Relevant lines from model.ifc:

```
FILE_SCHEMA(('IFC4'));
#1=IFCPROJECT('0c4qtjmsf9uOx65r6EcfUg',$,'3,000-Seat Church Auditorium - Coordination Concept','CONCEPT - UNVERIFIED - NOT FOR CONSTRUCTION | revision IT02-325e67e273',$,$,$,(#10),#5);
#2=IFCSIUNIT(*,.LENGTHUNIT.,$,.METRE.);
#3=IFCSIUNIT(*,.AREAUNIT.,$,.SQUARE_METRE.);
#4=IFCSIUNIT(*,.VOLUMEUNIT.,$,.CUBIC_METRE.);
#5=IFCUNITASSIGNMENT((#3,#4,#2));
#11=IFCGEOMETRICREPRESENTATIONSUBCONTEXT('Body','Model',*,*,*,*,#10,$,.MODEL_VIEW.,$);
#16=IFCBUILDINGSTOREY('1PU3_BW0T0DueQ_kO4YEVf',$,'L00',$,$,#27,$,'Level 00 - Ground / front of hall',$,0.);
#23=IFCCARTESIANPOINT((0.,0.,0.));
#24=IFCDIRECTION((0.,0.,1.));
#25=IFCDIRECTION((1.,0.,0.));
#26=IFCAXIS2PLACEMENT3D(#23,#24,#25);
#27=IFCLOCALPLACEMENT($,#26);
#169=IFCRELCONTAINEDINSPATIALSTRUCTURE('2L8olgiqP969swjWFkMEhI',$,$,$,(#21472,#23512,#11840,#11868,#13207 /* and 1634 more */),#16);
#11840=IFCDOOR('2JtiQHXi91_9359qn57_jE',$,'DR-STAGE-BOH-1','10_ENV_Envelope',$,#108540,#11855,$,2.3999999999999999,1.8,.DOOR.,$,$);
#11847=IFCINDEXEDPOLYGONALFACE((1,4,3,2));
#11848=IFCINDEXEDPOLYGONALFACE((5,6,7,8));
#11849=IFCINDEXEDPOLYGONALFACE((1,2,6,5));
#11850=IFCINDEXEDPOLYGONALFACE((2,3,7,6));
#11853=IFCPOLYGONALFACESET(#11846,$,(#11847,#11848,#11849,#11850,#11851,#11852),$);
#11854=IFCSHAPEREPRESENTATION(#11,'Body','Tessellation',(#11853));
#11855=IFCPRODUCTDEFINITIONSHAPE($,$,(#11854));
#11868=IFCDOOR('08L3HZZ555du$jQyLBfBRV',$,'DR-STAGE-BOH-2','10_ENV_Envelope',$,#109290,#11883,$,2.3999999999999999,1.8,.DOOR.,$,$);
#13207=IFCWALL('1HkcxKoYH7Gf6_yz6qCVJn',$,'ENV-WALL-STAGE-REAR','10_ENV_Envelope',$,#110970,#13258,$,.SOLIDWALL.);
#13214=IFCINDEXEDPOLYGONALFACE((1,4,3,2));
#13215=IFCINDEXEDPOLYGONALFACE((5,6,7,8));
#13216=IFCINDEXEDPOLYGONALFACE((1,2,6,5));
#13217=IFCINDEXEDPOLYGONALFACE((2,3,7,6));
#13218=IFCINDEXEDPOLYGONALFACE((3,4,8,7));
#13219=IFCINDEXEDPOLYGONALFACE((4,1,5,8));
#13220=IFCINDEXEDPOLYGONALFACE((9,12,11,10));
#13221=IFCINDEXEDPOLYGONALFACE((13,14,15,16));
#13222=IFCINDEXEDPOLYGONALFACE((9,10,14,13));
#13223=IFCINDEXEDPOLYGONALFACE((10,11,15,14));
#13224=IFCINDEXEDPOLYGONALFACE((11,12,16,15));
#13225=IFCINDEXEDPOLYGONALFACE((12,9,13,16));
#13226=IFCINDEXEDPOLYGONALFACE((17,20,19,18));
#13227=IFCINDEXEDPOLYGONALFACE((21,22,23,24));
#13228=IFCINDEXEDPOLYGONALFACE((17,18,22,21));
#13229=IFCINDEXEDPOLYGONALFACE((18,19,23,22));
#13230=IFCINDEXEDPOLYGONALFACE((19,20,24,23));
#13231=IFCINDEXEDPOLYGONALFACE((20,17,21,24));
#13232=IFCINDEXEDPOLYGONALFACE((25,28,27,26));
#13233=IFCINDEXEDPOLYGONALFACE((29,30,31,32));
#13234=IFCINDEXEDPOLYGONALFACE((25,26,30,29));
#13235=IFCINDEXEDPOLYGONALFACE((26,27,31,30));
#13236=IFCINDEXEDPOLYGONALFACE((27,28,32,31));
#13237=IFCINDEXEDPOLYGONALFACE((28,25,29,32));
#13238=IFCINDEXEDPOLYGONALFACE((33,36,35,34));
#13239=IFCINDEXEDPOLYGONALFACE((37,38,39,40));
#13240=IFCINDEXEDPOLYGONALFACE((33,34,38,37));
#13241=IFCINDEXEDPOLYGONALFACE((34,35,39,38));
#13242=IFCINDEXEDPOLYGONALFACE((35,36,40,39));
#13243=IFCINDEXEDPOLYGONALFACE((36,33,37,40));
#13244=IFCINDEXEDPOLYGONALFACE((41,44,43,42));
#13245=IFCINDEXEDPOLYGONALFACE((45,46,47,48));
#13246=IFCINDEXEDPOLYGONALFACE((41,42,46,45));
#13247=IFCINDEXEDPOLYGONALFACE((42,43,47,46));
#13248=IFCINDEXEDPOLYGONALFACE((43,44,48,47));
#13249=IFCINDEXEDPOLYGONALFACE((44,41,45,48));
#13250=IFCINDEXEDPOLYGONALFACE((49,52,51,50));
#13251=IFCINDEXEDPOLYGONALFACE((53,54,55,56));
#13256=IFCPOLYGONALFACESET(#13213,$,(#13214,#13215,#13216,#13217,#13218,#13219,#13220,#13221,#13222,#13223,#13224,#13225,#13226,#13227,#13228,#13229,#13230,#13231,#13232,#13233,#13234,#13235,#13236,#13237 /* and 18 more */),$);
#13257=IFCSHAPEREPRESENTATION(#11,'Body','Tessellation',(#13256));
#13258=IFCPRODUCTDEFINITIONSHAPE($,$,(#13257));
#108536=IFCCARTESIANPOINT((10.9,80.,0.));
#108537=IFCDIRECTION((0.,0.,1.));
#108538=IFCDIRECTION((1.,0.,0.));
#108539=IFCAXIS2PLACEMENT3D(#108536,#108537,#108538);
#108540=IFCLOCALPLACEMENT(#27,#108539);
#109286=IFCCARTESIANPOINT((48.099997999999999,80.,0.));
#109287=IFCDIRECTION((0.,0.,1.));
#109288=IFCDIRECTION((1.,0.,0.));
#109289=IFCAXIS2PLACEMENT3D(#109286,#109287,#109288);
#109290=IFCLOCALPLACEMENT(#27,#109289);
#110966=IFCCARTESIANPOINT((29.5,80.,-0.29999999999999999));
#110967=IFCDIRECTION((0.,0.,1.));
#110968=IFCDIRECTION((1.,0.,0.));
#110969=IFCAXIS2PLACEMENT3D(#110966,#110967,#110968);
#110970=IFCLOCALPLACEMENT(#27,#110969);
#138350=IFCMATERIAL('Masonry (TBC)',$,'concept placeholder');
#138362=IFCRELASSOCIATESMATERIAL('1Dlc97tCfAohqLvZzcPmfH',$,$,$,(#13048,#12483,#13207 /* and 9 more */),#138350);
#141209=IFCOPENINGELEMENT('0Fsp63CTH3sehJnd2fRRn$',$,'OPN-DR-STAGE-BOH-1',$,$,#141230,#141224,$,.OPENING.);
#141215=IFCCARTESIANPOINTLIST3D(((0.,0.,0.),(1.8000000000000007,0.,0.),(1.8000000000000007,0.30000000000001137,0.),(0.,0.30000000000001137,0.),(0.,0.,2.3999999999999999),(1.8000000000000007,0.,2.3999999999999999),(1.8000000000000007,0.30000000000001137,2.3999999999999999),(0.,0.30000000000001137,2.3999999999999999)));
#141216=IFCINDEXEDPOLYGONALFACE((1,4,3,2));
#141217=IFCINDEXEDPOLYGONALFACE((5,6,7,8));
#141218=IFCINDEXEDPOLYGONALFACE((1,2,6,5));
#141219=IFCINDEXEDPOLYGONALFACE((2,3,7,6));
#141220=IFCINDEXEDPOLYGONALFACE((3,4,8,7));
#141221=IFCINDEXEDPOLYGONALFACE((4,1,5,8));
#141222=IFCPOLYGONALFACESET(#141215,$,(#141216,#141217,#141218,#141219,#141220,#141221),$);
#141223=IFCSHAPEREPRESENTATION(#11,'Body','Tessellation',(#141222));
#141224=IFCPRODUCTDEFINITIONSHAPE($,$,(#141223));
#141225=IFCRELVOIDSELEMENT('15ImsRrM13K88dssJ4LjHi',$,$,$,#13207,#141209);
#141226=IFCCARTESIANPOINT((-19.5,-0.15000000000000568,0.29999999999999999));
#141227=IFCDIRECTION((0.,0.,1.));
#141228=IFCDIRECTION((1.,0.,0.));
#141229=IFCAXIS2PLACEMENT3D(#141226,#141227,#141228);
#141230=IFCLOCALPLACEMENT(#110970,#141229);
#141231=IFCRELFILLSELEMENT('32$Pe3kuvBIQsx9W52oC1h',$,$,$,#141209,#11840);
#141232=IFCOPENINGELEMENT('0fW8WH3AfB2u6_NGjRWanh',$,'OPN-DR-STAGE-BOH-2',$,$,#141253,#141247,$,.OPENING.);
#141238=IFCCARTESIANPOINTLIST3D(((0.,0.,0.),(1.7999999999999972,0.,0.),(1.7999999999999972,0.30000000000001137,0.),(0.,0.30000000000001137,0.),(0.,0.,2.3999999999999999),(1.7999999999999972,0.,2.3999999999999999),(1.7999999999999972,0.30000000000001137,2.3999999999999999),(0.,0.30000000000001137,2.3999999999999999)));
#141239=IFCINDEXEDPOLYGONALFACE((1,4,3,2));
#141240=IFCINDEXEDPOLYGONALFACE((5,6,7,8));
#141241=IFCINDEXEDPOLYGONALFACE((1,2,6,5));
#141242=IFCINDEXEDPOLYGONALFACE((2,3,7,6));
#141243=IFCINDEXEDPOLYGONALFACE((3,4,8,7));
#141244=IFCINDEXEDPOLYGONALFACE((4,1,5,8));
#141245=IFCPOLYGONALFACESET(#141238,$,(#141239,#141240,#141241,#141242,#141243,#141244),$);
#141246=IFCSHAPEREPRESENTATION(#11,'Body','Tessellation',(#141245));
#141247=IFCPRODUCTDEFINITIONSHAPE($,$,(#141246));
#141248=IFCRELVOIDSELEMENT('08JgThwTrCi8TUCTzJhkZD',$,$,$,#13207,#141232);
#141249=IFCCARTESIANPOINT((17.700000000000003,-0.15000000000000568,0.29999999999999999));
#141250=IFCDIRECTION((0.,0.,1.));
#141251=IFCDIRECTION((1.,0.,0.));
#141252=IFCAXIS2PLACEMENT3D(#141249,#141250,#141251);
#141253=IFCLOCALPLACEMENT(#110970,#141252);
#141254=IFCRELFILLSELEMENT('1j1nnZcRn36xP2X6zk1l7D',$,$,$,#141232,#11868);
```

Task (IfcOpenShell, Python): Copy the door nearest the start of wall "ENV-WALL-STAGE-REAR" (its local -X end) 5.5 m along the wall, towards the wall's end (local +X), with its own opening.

```python
import ifcopenshell
import ifcopenshell.api.feature
import ifcopenshell.api.geometry
import ifcopenshell.api.root
import ifcopenshell.geom
import ifcopenshell.util.element
import ifcopenshell.util.placement
import ifcopenshell.util.shape
import ifcopenshell.util.unit

model = ifcopenshell.open("model.ifc")
unit_scale = ifcopenshell.util.unit.calculate_unit_scale(model)
settings = ifcopenshell.geom.settings()


def volume(element):
    """Net volume in cubic metres, openings subtracted."""
    shape = ifcopenshell.geom.create_shape(settings, element)
    return ifcopenshell.util.shape.get_volume(shape.geometry)


door = model.by_guid("2JtiQHXi91_9359qn57_jE")
opening = door.FillsVoids[0].RelatingOpeningElement
wall = opening.VoidsElements[0].RelatingBuildingElement
before = volume(wall)
shift = ifcopenshell.util.placement.get_local_placement(wall.ObjectPlacement)[:3, 0] * 5.5 / unit_scale

# copy_class copies the void relationship, type, container and properties, but no geometry.
new_opening = ifcopenshell.api.root.copy_class(model, product=opening)
new_opening.Representation = ifcopenshell.util.element.copy_deep(
    model, opening.Representation, exclude=["IfcGeometricRepresentationContext", "IfcRepresentationMap"]
)
new_door = ifcopenshell.api.root.copy_class(model, product=door)
new_door.Representation = ifcopenshell.util.element.copy_deep(
    model, door.Representation, exclude=["IfcGeometricRepresentationContext", "IfcRepresentationMap"]
)
ifcopenshell.api.feature.add_filling(model, opening=new_opening, element=new_door)

for old, new in ((opening, new_opening), (door, new_door)):
    matrix = ifcopenshell.util.placement.get_local_placement(old.ObjectPlacement)
    matrix[:3, 3] += shift
    ifcopenshell.api.geometry.edit_object_placement(model, product=new, matrix=matrix, is_si=False)

after = volume(wall)

print(f"wall volume {before:.3f} -> {after:.3f} m3")

model.write("model_rev.ifc")
```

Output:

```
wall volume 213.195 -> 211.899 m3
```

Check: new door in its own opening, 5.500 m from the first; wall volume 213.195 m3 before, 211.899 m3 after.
